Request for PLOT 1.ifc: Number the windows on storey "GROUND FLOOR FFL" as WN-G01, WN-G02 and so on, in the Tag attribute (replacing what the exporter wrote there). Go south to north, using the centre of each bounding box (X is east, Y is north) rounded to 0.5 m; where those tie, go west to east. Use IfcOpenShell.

First a look at what the model holds.

```python
import ifcopenshell
import ifcopenshell.util.element
import ifcopenshell.util.placement

model = ifcopenshell.open("PLOT 1.ifc")
print(model.schema)
storey = next(s for s in model.by_type("IfcBuildingStorey") if s.Name == "GROUND FLOOR FFL")
windows = [e for e in ifcopenshell.util.element.get_decomposition(storey) if e.is_a("IfcWindow")]
for e in sorted(windows, key=lambda e: e.id()):
    origin = ifcopenshell.util.placement.get_local_placement(e.ObjectPlacement)[:3, 3]
    print(e.id(), e.Tag, e.Name, origin.round(2) + 0.0, sep=" | ")
```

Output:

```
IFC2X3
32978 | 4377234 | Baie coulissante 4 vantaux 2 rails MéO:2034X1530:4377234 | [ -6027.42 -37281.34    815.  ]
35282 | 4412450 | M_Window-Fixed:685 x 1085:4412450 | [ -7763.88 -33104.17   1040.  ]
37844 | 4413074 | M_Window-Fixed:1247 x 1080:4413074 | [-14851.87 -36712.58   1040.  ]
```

```python
import ifcopenshell
import ifcopenshell.geom
import ifcopenshell.util.element
import ifcopenshell.util.shape

model = ifcopenshell.open("PLOT 1.ifc")
settings = ifcopenshell.geom.settings()
settings.set("use-world-coords", True)


def centre(element):
    shape = ifcopenshell.geom.create_shape(settings, element)
    return ifcopenshell.util.shape.get_bbox_centroid(shape.geometry)


storey = next(s for s in model.by_type("IfcBuildingStorey") if s.Name == "GROUND FLOOR FFL")
windows = [e for e in ifcopenshell.util.element.get_decomposition(storey) if e.is_a("IfcWindow")]

# Insertion points can sit at a corner or the storey origin, so sort by the geometry (in metres).
centres = {e: centre(e) for e in windows}
windows.sort(key=lambda e: (round(centres[e][1] / 0.5), centres[e][0]))

for i, e in enumerate(windows, start=1):
    number = f"WN-G{i:02d}"
    e.Tag = number
    print(e.id(), number)

model.write("PLOT 1_edited.ifc")
```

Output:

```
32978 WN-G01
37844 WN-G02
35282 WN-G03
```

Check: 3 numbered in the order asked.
